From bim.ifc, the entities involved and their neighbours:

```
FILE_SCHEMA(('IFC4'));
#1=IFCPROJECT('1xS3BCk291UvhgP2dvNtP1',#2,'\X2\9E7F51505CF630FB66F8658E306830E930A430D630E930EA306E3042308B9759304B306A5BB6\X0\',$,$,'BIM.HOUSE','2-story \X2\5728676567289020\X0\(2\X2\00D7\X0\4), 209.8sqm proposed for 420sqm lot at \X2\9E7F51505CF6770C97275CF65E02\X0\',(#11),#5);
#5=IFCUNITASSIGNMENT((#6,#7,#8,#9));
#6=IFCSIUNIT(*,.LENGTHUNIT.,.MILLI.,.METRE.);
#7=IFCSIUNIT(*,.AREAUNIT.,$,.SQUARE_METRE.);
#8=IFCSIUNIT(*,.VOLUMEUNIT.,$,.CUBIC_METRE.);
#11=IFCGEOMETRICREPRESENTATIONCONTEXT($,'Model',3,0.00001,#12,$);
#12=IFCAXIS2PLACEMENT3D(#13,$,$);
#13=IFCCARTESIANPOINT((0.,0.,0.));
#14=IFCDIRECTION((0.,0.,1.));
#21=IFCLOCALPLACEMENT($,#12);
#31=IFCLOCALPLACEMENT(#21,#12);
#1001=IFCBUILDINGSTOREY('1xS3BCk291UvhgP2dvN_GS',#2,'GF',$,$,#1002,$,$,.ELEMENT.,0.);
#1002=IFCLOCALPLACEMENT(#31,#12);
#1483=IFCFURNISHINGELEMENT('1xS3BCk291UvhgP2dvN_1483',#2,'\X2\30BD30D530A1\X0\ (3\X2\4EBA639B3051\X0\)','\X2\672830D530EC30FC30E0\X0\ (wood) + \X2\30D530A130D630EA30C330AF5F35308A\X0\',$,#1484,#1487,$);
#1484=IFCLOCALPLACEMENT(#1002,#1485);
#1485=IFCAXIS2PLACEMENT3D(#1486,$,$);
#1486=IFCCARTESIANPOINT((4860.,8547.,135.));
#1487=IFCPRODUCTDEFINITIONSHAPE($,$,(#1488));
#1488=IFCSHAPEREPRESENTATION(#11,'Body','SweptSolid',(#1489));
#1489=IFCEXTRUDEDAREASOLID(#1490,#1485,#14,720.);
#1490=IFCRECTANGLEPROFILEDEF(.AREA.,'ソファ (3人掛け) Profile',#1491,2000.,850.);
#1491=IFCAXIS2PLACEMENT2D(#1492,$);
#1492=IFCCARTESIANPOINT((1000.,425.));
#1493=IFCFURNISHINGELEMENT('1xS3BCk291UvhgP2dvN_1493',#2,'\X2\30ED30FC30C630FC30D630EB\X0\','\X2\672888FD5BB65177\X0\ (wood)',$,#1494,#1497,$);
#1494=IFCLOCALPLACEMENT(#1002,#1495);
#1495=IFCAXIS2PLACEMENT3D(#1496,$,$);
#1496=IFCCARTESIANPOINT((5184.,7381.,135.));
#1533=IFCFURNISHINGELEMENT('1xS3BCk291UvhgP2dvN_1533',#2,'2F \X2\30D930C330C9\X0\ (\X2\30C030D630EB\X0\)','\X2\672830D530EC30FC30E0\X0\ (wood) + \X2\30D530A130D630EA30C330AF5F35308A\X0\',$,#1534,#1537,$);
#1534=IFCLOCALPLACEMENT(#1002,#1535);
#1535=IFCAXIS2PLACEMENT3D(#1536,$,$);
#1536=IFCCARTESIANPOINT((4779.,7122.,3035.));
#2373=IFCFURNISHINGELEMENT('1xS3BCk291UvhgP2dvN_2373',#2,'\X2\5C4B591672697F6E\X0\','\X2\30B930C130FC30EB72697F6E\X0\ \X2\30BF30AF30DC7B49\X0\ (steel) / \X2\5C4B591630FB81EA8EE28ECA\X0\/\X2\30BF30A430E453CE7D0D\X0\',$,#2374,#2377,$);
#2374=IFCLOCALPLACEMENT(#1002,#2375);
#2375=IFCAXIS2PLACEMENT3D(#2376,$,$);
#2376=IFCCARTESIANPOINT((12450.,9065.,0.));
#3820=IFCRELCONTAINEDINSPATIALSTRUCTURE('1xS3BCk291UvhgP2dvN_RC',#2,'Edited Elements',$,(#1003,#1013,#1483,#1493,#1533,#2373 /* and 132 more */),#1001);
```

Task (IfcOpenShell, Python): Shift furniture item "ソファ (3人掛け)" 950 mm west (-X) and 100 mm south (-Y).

```python
import ifcopenshell
import ifcopenshell.api.geometry
import ifcopenshell.util.placement

model = ifcopenshell.open("bim.ifc")

item = model.by_guid("1xS3BCk291UvhgP2dvN_1483")
matrix = ifcopenshell.util.placement.get_local_placement(item.ObjectPlacement)
matrix[0, 3] -= 950.0
matrix[1, 3] -= 100.0
ifcopenshell.api.geometry.edit_object_placement(model, product=item, matrix=matrix, is_si=False)

print(ifcopenshell.util.placement.get_local_placement(item.ObjectPlacement).round(3) + 0.0)

model.write("bim-out.ifc")
```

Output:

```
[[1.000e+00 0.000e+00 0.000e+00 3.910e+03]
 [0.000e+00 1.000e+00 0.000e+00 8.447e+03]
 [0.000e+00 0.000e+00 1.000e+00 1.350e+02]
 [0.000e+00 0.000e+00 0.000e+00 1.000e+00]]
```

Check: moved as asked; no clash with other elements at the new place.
